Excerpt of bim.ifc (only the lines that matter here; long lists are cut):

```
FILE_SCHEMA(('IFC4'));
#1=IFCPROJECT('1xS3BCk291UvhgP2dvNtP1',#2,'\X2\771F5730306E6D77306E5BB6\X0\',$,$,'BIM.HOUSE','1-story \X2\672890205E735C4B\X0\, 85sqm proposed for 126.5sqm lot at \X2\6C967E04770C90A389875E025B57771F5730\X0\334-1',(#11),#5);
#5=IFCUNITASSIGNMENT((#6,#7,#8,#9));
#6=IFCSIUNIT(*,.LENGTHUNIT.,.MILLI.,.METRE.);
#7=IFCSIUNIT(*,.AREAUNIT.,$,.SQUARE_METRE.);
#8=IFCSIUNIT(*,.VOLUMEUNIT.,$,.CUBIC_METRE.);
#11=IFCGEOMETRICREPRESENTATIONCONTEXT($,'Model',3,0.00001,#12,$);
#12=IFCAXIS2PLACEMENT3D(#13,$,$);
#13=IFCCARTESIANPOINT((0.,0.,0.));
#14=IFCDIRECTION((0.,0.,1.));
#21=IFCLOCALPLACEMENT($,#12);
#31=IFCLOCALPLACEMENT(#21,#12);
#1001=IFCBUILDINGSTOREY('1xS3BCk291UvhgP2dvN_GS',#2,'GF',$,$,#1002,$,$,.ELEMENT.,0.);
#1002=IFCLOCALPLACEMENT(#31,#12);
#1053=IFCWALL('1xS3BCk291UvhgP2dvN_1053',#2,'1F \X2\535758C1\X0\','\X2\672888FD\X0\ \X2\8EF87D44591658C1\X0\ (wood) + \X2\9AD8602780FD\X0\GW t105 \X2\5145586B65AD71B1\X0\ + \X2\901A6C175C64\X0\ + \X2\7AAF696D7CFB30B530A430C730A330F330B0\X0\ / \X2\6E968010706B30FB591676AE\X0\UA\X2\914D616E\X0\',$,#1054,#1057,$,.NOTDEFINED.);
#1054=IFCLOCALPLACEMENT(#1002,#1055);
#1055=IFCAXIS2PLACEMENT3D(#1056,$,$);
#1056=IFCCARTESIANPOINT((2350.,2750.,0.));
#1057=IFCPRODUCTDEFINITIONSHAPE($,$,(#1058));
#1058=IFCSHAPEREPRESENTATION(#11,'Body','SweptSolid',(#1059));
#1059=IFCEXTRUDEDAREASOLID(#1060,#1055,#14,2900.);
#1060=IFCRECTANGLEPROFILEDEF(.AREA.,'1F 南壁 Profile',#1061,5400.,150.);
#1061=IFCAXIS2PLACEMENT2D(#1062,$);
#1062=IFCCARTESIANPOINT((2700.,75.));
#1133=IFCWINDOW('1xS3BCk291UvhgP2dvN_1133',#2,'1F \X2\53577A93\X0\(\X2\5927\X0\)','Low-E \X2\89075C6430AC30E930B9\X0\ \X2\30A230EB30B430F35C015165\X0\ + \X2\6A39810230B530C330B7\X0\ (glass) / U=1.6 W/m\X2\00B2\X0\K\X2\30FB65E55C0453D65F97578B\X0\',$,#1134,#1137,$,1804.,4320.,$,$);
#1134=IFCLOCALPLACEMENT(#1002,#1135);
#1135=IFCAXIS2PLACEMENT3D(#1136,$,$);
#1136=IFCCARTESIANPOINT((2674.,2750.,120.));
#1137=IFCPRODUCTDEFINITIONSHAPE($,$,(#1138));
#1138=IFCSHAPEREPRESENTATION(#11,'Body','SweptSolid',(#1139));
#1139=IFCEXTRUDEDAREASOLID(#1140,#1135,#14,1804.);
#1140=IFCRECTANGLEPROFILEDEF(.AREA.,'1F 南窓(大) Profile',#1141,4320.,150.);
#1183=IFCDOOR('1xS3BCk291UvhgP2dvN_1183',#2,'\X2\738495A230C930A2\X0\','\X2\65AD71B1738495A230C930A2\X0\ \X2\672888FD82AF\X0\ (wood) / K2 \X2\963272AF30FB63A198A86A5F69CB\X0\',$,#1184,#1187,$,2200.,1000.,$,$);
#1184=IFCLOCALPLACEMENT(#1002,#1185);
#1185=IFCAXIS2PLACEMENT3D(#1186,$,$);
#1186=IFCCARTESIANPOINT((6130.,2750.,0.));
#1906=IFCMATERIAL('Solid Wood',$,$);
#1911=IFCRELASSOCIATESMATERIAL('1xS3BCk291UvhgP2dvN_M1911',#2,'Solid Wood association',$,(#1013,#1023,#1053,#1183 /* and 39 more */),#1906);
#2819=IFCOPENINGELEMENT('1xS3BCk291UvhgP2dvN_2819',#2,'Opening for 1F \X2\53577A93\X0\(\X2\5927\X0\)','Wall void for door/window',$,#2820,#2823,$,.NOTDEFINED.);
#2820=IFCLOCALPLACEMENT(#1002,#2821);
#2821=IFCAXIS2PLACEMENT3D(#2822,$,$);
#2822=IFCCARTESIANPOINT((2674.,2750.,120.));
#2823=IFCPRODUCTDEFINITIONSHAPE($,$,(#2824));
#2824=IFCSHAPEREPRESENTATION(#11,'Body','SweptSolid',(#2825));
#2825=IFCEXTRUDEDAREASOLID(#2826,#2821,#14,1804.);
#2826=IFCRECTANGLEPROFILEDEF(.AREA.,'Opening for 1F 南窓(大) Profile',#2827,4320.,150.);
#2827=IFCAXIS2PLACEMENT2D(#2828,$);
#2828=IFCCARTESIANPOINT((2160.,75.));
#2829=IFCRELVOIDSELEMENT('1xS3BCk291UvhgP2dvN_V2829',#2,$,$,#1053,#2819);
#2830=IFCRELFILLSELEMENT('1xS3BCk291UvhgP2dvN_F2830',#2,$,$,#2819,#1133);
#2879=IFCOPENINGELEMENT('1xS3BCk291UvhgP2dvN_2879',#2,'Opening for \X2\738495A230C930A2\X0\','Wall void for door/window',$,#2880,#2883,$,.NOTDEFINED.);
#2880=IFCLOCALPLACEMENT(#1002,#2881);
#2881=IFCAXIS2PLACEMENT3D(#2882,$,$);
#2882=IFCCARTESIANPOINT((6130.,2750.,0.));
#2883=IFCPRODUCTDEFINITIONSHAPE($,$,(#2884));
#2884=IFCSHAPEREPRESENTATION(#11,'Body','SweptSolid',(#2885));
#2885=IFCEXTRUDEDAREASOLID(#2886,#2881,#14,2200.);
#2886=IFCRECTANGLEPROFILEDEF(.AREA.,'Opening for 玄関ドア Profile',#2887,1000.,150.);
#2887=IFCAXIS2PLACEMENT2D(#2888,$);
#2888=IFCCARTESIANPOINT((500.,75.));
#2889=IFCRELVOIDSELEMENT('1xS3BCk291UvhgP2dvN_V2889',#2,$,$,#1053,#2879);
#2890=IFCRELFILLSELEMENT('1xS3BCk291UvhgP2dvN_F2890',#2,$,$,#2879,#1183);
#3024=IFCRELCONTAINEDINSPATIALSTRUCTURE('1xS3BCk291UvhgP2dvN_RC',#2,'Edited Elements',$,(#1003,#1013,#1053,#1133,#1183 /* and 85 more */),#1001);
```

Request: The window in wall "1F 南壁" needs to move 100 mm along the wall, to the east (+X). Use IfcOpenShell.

```python
import ifcopenshell
import ifcopenshell.api.geometry
import ifcopenshell.util.placement
import ifcopenshell.util.unit

model = ifcopenshell.open("bim.ifc")
unit_scale = ifcopenshell.util.unit.calculate_unit_scale(model)

window = model.by_guid("1xS3BCk291UvhgP2dvN_1133")
opening = window.FillsVoids[0].RelatingOpeningElement
wall = opening.VoidsElements[0].RelatingBuildingElement

wall_matrix = ifcopenshell.util.placement.get_local_placement(wall.ObjectPlacement)
shift = wall_matrix[:3, 0] * 0.1 / unit_scale
before = ifcopenshell.util.placement.get_local_placement(window.ObjectPlacement)[:3, 3].copy()

# The window is not placed relative to its opening, so move both.
for product in (opening, window):
    matrix = ifcopenshell.util.placement.get_local_placement(product.ObjectPlacement)
    matrix[:3, 3] += shift
    ifcopenshell.api.geometry.edit_object_placement(model, product=product, matrix=matrix, is_si=False)

after = ifcopenshell.util.placement.get_local_placement(window.ObjectPlacement)[:3, 3]
print("window moved by", (after - before).round(3) + 0.0)

model.write("bim_edited.ifc")
```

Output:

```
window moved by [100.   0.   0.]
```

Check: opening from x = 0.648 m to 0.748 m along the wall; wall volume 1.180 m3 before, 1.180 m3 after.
